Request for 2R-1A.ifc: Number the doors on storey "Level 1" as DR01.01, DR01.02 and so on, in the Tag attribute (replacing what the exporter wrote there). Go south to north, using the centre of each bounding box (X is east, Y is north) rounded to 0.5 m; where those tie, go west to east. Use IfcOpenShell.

First a look at what the model holds.

```python
import ifcopenshell
import ifcopenshell.util.element
import ifcopenshell.util.placement

model = ifcopenshell.open("2R-1A.ifc")
print(model.schema)
storey = next(s for s in model.by_type("IfcBuildingStorey") if s.Name == "Level 1")
doors = [e for e in ifcopenshell.util.element.get_decomposition(storey) if e.is_a("IfcDoor")]
for e in sorted(doors, key=lambda e: e.id()):
    origin = ifcopenshell.util.placement.get_local_placement(e.ObjectPlacement)[:3, 3]
    print(e.id(), e.Tag, e.Name, origin.round(2) + 0.0, sep=" | ")
```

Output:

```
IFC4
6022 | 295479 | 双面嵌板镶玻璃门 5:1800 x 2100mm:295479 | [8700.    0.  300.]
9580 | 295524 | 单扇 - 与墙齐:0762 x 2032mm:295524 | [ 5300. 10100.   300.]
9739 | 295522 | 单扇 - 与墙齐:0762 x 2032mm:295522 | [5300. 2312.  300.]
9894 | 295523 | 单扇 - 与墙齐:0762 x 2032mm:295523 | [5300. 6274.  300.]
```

```python
import ifcopenshell
import ifcopenshell.geom
import ifcopenshell.util.element
import ifcopenshell.util.shape

model = ifcopenshell.open("2R-1A.ifc")
settings = ifcopenshell.geom.settings()
settings.set("use-world-coords", True)


def centre(element):
    shape = ifcopenshell.geom.create_shape(settings, element)
    return ifcopenshell.util.shape.get_bbox_centroid(shape.geometry)


storey = next(s for s in model.by_type("IfcBuildingStorey") if s.Name == "Level 1")
doors = [e for e in ifcopenshell.util.element.get_decomposition(storey) if e.is_a("IfcDoor")]

# Insertion points can sit at a corner or the storey origin, so sort by the geometry (in metres).
centres = {e: centre(e) for e in doors}
doors.sort(key=lambda e: (round(centres[e][1] / 0.5), centres[e][0]))

for i, e in enumerate(doors, start=1):
    number = f"DR01.{i:02d}"
    e.Tag = number
    print(e.id(), number)

model.write("2R-1A-out.ifc")
```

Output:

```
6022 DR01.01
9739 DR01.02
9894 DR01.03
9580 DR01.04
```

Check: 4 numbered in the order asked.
